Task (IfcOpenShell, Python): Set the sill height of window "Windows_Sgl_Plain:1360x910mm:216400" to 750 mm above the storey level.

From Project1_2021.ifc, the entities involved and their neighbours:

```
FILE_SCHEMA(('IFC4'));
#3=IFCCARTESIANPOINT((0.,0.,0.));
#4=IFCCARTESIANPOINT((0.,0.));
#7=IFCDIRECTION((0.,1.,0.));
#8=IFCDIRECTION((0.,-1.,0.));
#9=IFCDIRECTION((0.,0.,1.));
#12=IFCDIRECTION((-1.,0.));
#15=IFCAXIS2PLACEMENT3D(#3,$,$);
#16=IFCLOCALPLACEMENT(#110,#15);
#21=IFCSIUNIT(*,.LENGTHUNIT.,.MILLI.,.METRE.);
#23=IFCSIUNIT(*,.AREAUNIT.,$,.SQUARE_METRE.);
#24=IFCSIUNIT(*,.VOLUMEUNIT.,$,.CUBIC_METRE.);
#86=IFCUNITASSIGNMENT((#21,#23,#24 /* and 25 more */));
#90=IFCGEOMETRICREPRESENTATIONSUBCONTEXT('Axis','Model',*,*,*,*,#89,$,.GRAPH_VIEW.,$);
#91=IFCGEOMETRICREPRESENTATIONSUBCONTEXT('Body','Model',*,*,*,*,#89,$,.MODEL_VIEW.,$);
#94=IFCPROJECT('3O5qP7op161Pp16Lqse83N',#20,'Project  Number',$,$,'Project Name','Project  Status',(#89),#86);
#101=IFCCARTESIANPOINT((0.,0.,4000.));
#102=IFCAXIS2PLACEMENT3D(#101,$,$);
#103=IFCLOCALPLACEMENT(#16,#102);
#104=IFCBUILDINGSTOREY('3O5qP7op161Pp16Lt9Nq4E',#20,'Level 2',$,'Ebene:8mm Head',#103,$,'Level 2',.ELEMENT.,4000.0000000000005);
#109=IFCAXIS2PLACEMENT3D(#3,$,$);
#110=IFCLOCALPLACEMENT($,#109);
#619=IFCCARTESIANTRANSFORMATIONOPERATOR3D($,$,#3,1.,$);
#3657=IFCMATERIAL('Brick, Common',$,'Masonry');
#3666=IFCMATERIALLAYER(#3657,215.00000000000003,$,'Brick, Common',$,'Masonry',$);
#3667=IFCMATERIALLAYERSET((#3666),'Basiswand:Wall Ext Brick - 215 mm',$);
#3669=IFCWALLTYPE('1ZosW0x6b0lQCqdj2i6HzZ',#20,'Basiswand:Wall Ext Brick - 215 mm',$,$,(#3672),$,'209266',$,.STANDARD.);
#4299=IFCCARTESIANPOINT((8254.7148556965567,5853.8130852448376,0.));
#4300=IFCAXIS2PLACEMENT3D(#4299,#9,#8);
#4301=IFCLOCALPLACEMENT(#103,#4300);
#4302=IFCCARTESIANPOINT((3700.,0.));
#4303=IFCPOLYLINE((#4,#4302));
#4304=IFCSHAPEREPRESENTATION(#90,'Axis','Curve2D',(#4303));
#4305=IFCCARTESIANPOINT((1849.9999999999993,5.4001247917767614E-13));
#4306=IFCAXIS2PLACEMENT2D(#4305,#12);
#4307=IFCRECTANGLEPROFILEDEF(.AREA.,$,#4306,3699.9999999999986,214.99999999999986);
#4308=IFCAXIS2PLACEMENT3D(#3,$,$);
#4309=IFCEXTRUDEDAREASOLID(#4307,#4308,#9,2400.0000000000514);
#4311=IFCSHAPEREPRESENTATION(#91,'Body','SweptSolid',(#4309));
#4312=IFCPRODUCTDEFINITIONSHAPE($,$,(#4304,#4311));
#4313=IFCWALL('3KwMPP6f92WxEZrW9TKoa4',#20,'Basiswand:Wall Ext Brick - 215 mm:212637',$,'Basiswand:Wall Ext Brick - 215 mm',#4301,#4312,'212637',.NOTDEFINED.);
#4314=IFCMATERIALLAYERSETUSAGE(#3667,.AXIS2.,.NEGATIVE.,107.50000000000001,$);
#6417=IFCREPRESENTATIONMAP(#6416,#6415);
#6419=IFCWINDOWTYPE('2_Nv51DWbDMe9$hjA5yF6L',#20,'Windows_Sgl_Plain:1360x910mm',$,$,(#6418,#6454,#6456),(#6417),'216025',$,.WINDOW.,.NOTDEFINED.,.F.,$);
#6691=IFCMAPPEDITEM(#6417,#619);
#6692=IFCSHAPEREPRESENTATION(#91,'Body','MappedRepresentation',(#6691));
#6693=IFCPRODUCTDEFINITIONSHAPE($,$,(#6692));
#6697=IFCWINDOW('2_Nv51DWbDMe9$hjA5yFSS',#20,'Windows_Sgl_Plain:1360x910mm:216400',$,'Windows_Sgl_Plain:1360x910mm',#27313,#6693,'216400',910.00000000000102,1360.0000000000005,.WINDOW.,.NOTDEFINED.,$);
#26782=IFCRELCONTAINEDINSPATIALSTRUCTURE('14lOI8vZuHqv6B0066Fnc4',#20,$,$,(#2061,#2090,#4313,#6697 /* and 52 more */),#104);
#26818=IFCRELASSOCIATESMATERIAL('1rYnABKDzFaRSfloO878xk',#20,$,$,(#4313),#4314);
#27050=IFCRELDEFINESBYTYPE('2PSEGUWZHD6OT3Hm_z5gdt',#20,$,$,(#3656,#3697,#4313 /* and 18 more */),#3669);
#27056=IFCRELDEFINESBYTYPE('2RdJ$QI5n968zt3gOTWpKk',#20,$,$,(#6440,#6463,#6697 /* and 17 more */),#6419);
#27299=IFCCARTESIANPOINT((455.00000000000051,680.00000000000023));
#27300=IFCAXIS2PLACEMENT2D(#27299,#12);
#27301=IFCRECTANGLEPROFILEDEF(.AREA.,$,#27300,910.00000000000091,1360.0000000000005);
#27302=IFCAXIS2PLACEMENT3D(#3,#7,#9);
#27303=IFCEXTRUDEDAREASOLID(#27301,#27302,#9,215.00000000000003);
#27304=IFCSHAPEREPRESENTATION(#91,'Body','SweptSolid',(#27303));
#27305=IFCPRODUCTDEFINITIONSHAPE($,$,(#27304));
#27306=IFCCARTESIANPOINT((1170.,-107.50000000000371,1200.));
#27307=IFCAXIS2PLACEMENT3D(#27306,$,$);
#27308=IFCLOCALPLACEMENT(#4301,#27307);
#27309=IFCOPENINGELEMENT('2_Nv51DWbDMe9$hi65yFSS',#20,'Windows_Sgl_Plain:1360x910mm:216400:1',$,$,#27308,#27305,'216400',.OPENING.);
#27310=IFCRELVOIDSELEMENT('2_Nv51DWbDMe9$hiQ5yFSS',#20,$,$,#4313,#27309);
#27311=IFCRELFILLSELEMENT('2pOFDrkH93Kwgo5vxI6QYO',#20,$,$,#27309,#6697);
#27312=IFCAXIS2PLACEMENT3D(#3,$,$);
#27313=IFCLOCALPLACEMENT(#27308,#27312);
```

```python
import numpy as np
import ifcopenshell
import ifcopenshell.api.geometry
import ifcopenshell.geom
import ifcopenshell.util.element
import ifcopenshell.util.placement
import ifcopenshell.util.shape
import ifcopenshell.util.unit

model = ifcopenshell.open("Project1_2021.ifc")
unit_scale = ifcopenshell.util.unit.calculate_unit_scale(model)

window = model.by_id(6697)
opening = window.FillsVoids[0].RelatingOpeningElement
storey = ifcopenshell.util.element.get_container(window, ifc_class="IfcBuildingStorey")
level = ifcopenshell.util.placement.get_local_placement(storey.ObjectPlacement)[2, 3]

# The opening's origin need not be at the sill, so measure its lowest point.
shape = ifcopenshell.geom.create_shape(ifcopenshell.geom.settings(), opening)
bottom = ifcopenshell.util.shape.get_shape_bottom_elevation(shape, shape.geometry) / unit_scale
dz = level + 750.0 - bottom

shift = np.array([0.0, 0.0, dz])
# The window is placed relative to its opening, so it follows when the opening moves.
matrix = ifcopenshell.util.placement.get_local_placement(opening.ObjectPlacement)
matrix[:3, 3] += shift
ifcopenshell.api.geometry.edit_object_placement(
    model, product=opening, matrix=matrix, is_si=False, should_transform_children=True
)

print(f"moved by {dz * unit_scale:+.3f} m")

model.write("Project1_2021_rev.ifc")
```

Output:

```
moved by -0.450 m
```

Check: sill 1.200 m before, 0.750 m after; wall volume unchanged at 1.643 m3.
